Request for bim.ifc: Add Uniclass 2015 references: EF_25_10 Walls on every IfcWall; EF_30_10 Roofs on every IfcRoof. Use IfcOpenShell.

First a look at what the model holds.

```python
import ifcopenshell

model = ifcopenshell.open("bim.ifc")
print(model.schema)
print("classifications:", [c.Name for c in model.by_type("IfcClassification")])
for ifc_class in ("IfcDoor", "IfcRoof", "IfcStair", "IfcWall", "IfcWindow"):
    print(ifc_class, len(model.by_type(ifc_class)))
```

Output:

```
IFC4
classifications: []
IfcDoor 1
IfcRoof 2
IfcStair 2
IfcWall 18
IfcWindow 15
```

```python
import ifcopenshell
import ifcopenshell.api.classification

model = ifcopenshell.open("bim.ifc")

system = ifcopenshell.api.classification.add_classification(model, classification="Uniclass 2015")

codes = {
    "IfcWall": ("EF_25_10", "Walls"),
    "IfcRoof": ("EF_30_10", "Roofs"),
}
for ifc_class, (code, name) in codes.items():
    products = model.by_type(ifc_class)
    ifcopenshell.api.classification.add_reference(
        model, products=products, classification=system, identification=code, name=name
    )
    print(code, len(products))

model.write("bim_v2.ifc")
```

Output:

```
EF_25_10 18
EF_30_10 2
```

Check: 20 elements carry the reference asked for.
